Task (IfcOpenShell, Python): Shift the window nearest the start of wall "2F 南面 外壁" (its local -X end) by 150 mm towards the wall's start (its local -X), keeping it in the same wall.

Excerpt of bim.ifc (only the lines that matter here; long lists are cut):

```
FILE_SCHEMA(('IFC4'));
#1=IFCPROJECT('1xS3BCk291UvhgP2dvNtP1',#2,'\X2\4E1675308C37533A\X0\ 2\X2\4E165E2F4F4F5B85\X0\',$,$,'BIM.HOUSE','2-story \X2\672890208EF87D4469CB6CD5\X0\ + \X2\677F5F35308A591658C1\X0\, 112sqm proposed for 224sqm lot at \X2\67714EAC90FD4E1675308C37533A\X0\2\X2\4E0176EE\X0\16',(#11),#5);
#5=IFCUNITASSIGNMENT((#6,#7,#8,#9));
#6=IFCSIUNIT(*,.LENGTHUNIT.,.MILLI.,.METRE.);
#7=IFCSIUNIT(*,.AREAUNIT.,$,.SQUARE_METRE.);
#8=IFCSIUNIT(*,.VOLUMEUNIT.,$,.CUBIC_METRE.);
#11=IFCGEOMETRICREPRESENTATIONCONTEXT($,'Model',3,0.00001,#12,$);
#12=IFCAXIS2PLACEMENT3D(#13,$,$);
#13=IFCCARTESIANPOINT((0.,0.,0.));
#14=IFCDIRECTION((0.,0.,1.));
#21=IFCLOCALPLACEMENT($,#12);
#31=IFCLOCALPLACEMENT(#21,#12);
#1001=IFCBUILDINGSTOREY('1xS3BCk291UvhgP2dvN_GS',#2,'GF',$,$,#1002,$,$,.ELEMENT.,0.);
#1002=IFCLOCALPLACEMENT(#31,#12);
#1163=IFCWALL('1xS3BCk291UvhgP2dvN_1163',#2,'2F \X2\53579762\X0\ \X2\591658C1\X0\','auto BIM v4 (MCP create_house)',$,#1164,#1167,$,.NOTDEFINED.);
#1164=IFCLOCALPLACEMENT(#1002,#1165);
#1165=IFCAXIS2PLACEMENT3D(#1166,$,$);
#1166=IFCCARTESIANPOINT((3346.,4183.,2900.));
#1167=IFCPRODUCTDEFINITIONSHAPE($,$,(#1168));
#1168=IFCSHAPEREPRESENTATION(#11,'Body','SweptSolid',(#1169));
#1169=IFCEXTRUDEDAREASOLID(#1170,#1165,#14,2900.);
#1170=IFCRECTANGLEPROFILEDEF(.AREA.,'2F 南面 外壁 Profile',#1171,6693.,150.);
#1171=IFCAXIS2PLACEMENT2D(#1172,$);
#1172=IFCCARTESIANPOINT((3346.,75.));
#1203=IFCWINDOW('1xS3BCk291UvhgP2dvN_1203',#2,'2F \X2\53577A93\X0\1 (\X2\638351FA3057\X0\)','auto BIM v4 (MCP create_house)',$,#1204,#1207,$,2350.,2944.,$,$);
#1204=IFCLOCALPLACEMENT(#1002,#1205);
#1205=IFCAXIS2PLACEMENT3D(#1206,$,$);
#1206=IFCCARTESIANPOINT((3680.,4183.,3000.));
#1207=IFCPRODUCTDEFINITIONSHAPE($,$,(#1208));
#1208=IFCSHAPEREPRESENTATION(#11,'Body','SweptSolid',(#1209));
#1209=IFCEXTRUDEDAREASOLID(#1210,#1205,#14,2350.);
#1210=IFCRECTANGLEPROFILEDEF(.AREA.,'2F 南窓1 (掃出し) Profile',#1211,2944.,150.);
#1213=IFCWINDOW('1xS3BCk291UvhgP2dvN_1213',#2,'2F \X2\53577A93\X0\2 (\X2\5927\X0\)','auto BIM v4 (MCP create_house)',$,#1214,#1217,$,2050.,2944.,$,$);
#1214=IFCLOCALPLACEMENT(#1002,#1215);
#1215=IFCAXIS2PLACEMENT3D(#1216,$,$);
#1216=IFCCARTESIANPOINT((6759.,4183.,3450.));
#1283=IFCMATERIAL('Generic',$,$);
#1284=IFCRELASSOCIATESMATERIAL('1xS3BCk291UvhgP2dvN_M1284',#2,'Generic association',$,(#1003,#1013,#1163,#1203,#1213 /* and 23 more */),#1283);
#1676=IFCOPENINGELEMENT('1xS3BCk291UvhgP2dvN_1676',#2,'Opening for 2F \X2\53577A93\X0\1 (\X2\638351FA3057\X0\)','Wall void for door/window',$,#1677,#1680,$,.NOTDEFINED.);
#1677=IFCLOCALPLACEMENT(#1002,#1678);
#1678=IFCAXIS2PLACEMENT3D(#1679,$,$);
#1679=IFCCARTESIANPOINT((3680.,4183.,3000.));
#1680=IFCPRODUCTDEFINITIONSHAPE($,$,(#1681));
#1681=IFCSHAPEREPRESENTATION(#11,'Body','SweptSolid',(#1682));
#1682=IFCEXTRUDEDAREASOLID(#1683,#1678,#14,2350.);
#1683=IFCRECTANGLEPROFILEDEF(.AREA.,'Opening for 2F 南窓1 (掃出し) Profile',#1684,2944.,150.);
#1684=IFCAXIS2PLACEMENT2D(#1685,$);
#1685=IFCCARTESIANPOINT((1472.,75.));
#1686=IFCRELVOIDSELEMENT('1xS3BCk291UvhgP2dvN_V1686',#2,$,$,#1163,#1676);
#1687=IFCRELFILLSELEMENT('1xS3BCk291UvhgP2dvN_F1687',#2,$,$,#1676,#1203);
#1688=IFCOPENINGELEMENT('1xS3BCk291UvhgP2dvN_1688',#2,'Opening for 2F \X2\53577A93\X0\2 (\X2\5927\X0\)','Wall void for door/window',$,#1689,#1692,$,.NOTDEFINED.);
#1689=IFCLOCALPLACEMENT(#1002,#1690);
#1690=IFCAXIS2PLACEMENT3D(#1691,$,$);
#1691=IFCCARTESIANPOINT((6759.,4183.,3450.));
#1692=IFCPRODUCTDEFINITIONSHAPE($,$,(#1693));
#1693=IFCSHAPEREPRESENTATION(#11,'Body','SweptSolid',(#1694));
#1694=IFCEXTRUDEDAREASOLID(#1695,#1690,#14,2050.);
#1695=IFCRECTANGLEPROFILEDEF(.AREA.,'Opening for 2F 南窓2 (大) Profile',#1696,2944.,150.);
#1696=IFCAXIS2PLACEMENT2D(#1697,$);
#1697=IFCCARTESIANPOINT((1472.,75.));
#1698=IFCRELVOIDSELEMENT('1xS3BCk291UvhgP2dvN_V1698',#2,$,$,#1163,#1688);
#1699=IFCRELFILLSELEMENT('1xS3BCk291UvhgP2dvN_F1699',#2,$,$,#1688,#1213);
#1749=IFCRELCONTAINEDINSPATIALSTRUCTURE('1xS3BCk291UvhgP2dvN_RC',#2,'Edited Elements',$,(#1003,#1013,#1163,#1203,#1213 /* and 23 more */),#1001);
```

```python
import ifcopenshell
import ifcopenshell.api.geometry
import ifcopenshell.util.placement

model = ifcopenshell.open("bim.ifc")

window = model.by_id(1203)
opening = window.FillsVoids[0].RelatingOpeningElement
wall = opening.VoidsElements[0].RelatingBuildingElement

wall_matrix = ifcopenshell.util.placement.get_local_placement(wall.ObjectPlacement)
shift = wall_matrix[:3, 0] * -150.0
before = ifcopenshell.util.placement.get_local_placement(window.ObjectPlacement)[:3, 3].copy()

# The window is not placed relative to its opening, so move both.
for product in (opening, window):
    matrix = ifcopenshell.util.placement.get_local_placement(product.ObjectPlacement)
    matrix[:3, 3] += shift
    ifcopenshell.api.geometry.edit_object_placement(model, product=product, matrix=matrix, is_si=False)

after = ifcopenshell.util.placement.get_local_placement(window.ObjectPlacement)[:3, 3]
print("window moved by", (after - before).round(3) + 0.0)

model.write("bim_edited.ifc")
```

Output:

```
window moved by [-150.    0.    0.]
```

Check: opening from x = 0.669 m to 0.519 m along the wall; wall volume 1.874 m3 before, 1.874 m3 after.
